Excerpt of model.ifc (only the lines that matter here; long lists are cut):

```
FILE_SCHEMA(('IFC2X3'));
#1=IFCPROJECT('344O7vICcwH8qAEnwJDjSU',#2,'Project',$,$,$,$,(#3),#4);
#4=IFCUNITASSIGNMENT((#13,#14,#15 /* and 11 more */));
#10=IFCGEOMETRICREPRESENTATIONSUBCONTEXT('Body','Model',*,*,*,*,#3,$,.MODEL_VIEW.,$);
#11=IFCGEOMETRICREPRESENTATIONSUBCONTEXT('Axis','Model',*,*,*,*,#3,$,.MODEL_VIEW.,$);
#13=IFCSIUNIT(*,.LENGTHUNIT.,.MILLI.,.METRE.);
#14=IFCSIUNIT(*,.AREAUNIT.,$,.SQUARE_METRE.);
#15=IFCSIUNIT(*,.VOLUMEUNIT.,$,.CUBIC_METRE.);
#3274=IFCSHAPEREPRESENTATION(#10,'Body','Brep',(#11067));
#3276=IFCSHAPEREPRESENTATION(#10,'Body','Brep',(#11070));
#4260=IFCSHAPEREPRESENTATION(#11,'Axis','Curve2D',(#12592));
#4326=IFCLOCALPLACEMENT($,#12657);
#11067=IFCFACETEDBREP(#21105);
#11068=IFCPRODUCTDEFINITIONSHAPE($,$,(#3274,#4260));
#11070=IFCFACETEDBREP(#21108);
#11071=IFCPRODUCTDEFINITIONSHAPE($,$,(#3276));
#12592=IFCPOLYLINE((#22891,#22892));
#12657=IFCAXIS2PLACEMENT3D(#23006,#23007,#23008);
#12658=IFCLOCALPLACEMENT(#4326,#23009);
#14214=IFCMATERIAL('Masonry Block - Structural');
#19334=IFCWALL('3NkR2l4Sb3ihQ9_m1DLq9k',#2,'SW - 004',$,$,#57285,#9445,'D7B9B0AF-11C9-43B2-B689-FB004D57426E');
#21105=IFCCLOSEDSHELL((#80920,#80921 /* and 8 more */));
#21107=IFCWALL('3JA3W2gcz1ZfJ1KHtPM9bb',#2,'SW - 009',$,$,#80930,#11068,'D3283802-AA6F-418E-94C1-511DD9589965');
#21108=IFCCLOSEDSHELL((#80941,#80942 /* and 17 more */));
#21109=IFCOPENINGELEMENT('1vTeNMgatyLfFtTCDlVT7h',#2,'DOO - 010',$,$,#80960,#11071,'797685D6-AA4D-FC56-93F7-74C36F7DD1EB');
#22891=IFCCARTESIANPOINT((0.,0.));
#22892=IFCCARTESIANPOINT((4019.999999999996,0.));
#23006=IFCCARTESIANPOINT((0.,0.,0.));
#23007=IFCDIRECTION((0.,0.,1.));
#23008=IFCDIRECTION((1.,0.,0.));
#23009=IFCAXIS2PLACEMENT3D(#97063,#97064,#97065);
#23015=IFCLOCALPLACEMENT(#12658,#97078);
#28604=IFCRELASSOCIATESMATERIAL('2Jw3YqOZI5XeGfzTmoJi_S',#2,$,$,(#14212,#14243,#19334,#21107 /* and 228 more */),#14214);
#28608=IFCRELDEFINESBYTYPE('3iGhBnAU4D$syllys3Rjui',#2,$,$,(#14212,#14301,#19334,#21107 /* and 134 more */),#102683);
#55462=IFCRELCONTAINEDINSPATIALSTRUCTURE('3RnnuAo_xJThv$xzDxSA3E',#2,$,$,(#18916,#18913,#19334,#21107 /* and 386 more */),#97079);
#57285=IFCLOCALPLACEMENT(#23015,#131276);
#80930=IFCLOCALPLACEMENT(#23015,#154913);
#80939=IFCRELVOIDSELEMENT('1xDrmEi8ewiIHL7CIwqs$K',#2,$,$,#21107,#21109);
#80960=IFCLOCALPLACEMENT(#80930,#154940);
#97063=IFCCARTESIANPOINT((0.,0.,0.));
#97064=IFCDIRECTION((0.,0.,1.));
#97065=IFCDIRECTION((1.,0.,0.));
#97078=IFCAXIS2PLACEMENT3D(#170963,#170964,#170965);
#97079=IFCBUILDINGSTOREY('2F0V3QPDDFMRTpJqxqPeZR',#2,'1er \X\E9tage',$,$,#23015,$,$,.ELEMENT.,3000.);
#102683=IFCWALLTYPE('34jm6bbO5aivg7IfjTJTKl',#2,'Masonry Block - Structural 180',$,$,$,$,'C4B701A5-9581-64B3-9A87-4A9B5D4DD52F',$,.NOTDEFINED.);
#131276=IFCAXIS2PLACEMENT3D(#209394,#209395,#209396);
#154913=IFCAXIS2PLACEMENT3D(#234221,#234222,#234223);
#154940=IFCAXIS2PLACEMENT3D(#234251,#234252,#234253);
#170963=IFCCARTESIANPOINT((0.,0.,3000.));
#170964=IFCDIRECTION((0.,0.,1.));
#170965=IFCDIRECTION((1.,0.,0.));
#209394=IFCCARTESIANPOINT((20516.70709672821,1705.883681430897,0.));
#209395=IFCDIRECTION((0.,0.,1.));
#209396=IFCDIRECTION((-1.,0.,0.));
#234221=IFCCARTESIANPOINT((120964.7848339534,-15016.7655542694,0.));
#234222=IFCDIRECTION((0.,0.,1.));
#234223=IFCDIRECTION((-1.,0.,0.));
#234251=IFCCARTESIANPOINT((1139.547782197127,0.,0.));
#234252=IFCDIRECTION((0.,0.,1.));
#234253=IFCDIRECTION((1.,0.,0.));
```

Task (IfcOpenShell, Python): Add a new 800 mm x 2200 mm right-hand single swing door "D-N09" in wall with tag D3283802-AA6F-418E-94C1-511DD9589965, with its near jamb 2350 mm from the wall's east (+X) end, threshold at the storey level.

```python
import numpy as np
import ifcopenshell
import ifcopenshell.api.feature
import ifcopenshell.api.geometry
import ifcopenshell.api.root
import ifcopenshell.api.spatial
import ifcopenshell.api.type
import ifcopenshell.geom
import ifcopenshell.util.element
import ifcopenshell.util.placement
import ifcopenshell.util.representation
import ifcopenshell.util.shape
import ifcopenshell.util.unit

model = ifcopenshell.open("model.ifc")
unit_scale = ifcopenshell.util.unit.calculate_unit_scale(model)
settings = ifcopenshell.geom.settings()


def volume(element):
    """Net volume in cubic metres, openings subtracted."""
    shape = ifcopenshell.geom.create_shape(settings, element)
    return ifcopenshell.util.shape.get_volume(shape.geometry)


wall = model.by_guid("3JA3W2gcz1ZfJ1KHtPM9bb")
storey = ifcopenshell.util.element.get_container(wall, ifc_class="IfcBuildingStorey")
context = ifcopenshell.util.representation.get_context(model, "Model", "Body", "MODEL_VIEW")
before = volume(wall)

width, height, from_end, sill = 0.8, 2.2, 2.35, 0.0  # metres

# The wall runs along its own X axis, and the end named is its -X end.
wall_shape = ifcopenshell.geom.create_shape(settings, wall)
x, y, z = ifcopenshell.util.shape.get_vertices(wall_shape.geometry).T
start = x.min() + from_end
face, thickness = float(y.min()), float(y.max() - y.min())
wall_matrix = ifcopenshell.util.placement.get_local_placement(wall.ObjectPlacement)
level = ifcopenshell.util.placement.get_local_placement(storey.ObjectPlacement)[2, 3]


def in_wall(x, y):
    """Placement at x, y metres in the wall's axes, at sill height."""
    matrix = wall_matrix.copy()
    matrix[:, 3] = wall_matrix @ np.array([x / unit_scale, y / unit_scale, 0.0, 1.0])
    matrix[2, 3] = level + sill / unit_scale
    return matrix


# Opening: a box that overshoots both wall faces by 50 mm.
opening = ifcopenshell.api.root.create_entity(model, ifc_class="IfcOpeningElement")
box = ifcopenshell.api.geometry.add_wall_representation(
    model, context=context, length=width, height=height, thickness=thickness + 0.1
)
ifcopenshell.api.geometry.assign_representation(model, product=opening, representation=box)
ifcopenshell.api.geometry.edit_object_placement(model, product=opening, matrix=in_wall(start, face - 0.05), is_si=False)
ifcopenshell.api.feature.add_feature(model, feature=opening, element=wall)

door = ifcopenshell.api.root.create_entity(model, ifc_class="IfcDoor", name="D-N09")
door.OverallWidth, door.OverallHeight = width / unit_scale, height / unit_scale
body = ifcopenshell.api.geometry.add_door_representation(
    model,
    context=context,
    overall_width=door.OverallWidth,
    overall_height=door.OverallHeight,
    operation_type="SINGLE_SWING_RIGHT",
    lining_properties={"LiningDepth": thickness / unit_scale, "ThresholdDepth": thickness / unit_scale},
)
ifcopenshell.api.geometry.assign_representation(model, product=door, representation=body)
ifcopenshell.api.spatial.assign_container(model, products=[door], relating_structure=storey)
fills = ifcopenshell.api.feature.add_filling(model, opening=opening, element=door)
fills.OwnerHistory = door.OwnerHistory  # required in IFC2X3

# IFC2X3 keeps the operation on the door style.
style = ifcopenshell.api.root.create_entity(model, ifc_class="IfcDoorStyle", name="D-N09")
style.OperationType, style.ConstructionType = "SINGLE_SWING_RIGHT", "NOTDEFINED"
style.ParameterTakesPrecedence = style.Sizeable = False
ifcopenshell.api.type.assign_type(model, related_objects=[door], relating_type=style)

# The lining spans the wall, so the door starts at the wall face.
ifcopenshell.api.geometry.edit_object_placement(model, product=door, matrix=in_wall(start, face), is_si=False)

after = volume(wall)

print(f"wall volume {before:.3f} -> {after:.3f} m3")

model.write("model_updated.ifc")
```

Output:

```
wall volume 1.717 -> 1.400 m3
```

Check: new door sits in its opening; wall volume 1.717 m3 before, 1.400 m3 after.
